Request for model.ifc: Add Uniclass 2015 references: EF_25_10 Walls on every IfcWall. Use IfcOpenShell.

First a look at what the model holds.

```python
import ifcopenshell

model = ifcopenshell.open("model.ifc")
print(model.schema)
print("classifications:", [c.Name for c in model.by_type("IfcClassification")])
for ifc_class in ("IfcDoor", "IfcRoof", "IfcStair", "IfcWall", "IfcWindow"):
    print(ifc_class, len(model.by_type(ifc_class)))
```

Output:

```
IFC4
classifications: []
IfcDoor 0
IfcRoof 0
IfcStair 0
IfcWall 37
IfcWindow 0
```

```python
import ifcopenshell
import ifcopenshell.api.classification

model = ifcopenshell.open("model.ifc")

system = ifcopenshell.api.classification.add_classification(model, classification="Uniclass 2015")

codes = {
    "IfcWall": ("EF_25_10", "Walls"),
}
for ifc_class, (code, name) in codes.items():
    products = model.by_type(ifc_class)
    ifcopenshell.api.classification.add_reference(
        model, products=products, classification=system, identification=code, name=name
    )
    print(code, len(products))

model.write("model-out.ifc")
```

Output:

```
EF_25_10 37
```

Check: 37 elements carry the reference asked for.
